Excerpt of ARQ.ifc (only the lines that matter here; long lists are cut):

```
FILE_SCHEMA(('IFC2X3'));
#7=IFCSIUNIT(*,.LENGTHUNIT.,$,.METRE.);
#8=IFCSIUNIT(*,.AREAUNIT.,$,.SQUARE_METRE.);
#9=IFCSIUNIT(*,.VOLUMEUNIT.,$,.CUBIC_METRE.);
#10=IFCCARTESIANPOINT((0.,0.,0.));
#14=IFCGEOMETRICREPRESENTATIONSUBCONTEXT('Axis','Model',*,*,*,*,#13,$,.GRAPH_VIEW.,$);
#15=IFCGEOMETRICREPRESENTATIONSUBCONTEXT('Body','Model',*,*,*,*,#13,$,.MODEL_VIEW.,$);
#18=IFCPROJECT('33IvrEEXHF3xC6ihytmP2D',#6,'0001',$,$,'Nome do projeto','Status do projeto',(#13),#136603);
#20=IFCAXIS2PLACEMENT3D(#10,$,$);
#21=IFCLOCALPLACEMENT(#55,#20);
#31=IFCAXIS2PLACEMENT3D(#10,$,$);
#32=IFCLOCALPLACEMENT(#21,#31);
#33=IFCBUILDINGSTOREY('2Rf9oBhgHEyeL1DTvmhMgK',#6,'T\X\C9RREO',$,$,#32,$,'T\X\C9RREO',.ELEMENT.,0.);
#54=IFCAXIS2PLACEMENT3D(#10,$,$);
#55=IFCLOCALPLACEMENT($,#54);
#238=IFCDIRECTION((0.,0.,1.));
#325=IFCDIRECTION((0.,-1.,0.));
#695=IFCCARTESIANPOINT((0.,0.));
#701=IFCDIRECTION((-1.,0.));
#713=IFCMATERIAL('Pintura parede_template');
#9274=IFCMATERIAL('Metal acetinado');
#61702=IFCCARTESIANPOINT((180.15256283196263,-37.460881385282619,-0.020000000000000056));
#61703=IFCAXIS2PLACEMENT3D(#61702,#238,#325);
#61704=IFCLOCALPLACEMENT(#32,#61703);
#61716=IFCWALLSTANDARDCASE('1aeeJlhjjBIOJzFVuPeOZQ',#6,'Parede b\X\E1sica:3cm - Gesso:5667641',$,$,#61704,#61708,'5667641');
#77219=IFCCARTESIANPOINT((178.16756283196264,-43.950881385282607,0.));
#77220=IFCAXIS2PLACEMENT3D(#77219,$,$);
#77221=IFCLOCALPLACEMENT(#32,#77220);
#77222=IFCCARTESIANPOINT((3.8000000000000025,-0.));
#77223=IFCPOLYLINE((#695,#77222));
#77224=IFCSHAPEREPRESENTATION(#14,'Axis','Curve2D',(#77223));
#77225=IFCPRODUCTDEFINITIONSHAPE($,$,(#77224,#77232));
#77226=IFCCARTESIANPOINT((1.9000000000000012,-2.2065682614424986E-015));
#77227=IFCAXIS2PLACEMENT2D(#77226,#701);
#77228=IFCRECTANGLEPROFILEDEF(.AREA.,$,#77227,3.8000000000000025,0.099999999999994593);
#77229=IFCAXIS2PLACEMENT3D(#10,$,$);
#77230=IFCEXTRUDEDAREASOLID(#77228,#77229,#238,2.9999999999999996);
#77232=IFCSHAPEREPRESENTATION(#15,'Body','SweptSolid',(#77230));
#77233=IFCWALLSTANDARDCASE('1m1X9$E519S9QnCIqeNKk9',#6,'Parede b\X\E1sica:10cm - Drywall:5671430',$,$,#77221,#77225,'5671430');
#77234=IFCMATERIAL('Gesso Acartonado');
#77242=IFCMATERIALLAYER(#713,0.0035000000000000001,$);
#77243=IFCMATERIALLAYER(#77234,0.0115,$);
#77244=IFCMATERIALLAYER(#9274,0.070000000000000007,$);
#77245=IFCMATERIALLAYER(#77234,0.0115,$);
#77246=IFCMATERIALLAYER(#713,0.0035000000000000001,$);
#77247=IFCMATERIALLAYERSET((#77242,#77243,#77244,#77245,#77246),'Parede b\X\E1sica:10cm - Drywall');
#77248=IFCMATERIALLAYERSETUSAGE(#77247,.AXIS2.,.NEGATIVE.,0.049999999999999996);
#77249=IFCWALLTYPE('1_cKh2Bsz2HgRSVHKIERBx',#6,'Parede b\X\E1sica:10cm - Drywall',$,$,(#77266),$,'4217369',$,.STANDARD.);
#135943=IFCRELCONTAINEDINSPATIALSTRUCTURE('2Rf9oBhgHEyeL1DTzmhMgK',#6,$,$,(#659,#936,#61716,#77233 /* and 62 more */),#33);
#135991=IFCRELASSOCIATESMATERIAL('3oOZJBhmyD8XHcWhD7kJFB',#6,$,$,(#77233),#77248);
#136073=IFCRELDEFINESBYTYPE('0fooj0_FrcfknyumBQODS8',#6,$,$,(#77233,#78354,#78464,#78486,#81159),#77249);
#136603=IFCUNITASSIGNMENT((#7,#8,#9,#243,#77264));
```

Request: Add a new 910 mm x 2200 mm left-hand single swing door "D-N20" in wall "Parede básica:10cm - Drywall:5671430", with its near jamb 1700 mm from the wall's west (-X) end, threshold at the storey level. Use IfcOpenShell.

```python
import numpy as np
import ifcopenshell
import ifcopenshell.api.feature
import ifcopenshell.api.geometry
import ifcopenshell.api.root
import ifcopenshell.api.spatial
import ifcopenshell.api.type
import ifcopenshell.geom
import ifcopenshell.util.element
import ifcopenshell.util.placement
import ifcopenshell.util.representation
import ifcopenshell.util.shape
import ifcopenshell.util.unit

model = ifcopenshell.open("ARQ.ifc")
unit_scale = ifcopenshell.util.unit.calculate_unit_scale(model)
settings = ifcopenshell.geom.settings()


def volume(element):
    """Net volume in cubic metres, openings subtracted."""
    shape = ifcopenshell.geom.create_shape(settings, element)
    return ifcopenshell.util.shape.get_volume(shape.geometry)


wall = model.by_guid("1m1X9$E519S9QnCIqeNKk9")
storey = ifcopenshell.util.element.get_container(wall, ifc_class="IfcBuildingStorey")
context = ifcopenshell.util.representation.get_context(model, "Model", "Body", "MODEL_VIEW")
before = volume(wall)

width, height, from_end, sill = 0.91, 2.2, 1.7, 0.0  # metres

# The wall runs along its own X axis, and the end named is its -X end.
wall_shape = ifcopenshell.geom.create_shape(settings, wall)
x, y, z = ifcopenshell.util.shape.get_vertices(wall_shape.geometry).T
start = x.min() + from_end
face, thickness = float(y.min()), float(y.max() - y.min())
wall_matrix = ifcopenshell.util.placement.get_local_placement(wall.ObjectPlacement)
level = ifcopenshell.util.placement.get_local_placement(storey.ObjectPlacement)[2, 3]


def in_wall(x, y):
    """Placement at x, y metres in the wall's axes, at sill height."""
    matrix = wall_matrix.copy()
    matrix[:, 3] = wall_matrix @ np.array([x / unit_scale, y / unit_scale, 0.0, 1.0])
    matrix[2, 3] = level + sill / unit_scale
    return matrix


# Opening: a box that overshoots both wall faces by 50 mm.
opening = ifcopenshell.api.root.create_entity(model, ifc_class="IfcOpeningElement")
box = ifcopenshell.api.geometry.add_wall_representation(
    model, context=context, length=width, height=height, thickness=thickness + 0.1
)
ifcopenshell.api.geometry.assign_representation(model, product=opening, representation=box)
ifcopenshell.api.geometry.edit_object_placement(model, product=opening, matrix=in_wall(start, face - 0.05), is_si=False)
ifcopenshell.api.feature.add_feature(model, feature=opening, element=wall)

door = ifcopenshell.api.root.create_entity(model, ifc_class="IfcDoor", name="D-N20")
door.OverallWidth, door.OverallHeight = width / unit_scale, height / unit_scale
body = ifcopenshell.api.geometry.add_door_representation(
    model,
    context=context,
    overall_width=door.OverallWidth,
    overall_height=door.OverallHeight,
    operation_type="SINGLE_SWING_LEFT",
    lining_properties={"LiningDepth": thickness / unit_scale, "ThresholdDepth": thickness / unit_scale},
)
ifcopenshell.api.geometry.assign_representation(model, product=door, representation=body)
ifcopenshell.api.spatial.assign_container(model, products=[door], relating_structure=storey)
fills = ifcopenshell.api.feature.add_filling(model, opening=opening, element=door)
fills.OwnerHistory = door.OwnerHistory  # required in IFC2X3

# IFC2X3 keeps the operation on the door style.
style = ifcopenshell.api.root.create_entity(model, ifc_class="IfcDoorStyle", name="D-N20")
style.OperationType, style.ConstructionType = "SINGLE_SWING_LEFT", "NOTDEFINED"
style.ParameterTakesPrecedence = style.Sizeable = False
ifcopenshell.api.type.assign_type(model, related_objects=[door], relating_type=style)

# The lining spans the wall, so the door starts at the wall face.
ifcopenshell.api.geometry.edit_object_placement(model, product=door, matrix=in_wall(start, face), is_si=False)

after = volume(wall)

print(f"wall volume {before:.3f} -> {after:.3f} m3")

model.write("ARQ-out.ifc")
```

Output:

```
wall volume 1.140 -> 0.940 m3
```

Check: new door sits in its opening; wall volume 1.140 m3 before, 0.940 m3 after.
